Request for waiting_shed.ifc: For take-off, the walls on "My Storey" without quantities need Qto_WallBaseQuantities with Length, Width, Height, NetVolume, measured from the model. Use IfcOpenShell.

First a look at what the model holds.

```python
import ifcopenshell
import ifcopenshell.util.element
import ifcopenshell.util.unit

model = ifcopenshell.open("waiting_shed.ifc")
print(model.schema)
for unit_type in ("LENGTHUNIT", "AREAUNIT", "VOLUMEUNIT"):
    print(unit_type, ifcopenshell.util.unit.calculate_unit_scale(model, unit_type))
storey = next(s for s in model.by_type("IfcBuildingStorey") if s.Name == "My Storey")
walls = [e for e in ifcopenshell.util.element.get_decomposition(storey) if e.is_a("IfcWall")]
for e in sorted(walls, key=lambda e: e.id()):
    print(e.id(), e.is_a(), e.Name, list(ifcopenshell.util.element.get_psets(e, qtos_only=True)), sep=" | ")
```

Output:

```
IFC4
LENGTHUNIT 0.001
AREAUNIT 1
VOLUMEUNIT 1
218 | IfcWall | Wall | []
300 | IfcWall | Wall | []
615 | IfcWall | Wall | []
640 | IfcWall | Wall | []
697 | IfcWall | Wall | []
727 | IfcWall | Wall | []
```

```python
import ifcopenshell
import ifcopenshell.api.pset
import ifcopenshell.geom
import ifcopenshell.util.element
import ifcopenshell.util.shape
import ifcopenshell.util.unit

model = ifcopenshell.open("waiting_shed.ifc")
unit_scale = ifcopenshell.util.unit.calculate_unit_scale(model)
volume_scale = ifcopenshell.util.unit.calculate_unit_scale(model, "VOLUMEUNIT")
settings = ifcopenshell.geom.settings()

storey = next(s for s in model.by_type("IfcBuildingStorey") if s.Name == "My Storey")
walls = [e for e in ifcopenshell.util.element.get_decomposition(storey) if e.is_a("IfcWall")]

for e in sorted(walls, key=lambda e: e.id()):
    if ifcopenshell.util.element.get_psets(e, qtos_only=True, should_inherit=False):
        continue
    # Geometry comes back in metres, in the element's own axes.
    shape = ifcopenshell.geom.create_shape(settings, e)
    values = {
        "Length": ifcopenshell.util.shape.get_x(shape.geometry) / unit_scale,
        "Width": ifcopenshell.util.shape.get_y(shape.geometry) / unit_scale,
        "Height": ifcopenshell.util.shape.get_z(shape.geometry) / unit_scale,
        "NetVolume": ifcopenshell.util.shape.get_volume(shape.geometry) / volume_scale,
    }
    qto = ifcopenshell.api.pset.add_qto(model, product=e, name="Qto_WallBaseQuantities")
    ifcopenshell.api.pset.edit_qto(model, qto=qto, properties=values)
    print(e.id(), {k: round(v, 3) for k, v in values.items()})

model.write("waiting_shed_v2.ifc")
```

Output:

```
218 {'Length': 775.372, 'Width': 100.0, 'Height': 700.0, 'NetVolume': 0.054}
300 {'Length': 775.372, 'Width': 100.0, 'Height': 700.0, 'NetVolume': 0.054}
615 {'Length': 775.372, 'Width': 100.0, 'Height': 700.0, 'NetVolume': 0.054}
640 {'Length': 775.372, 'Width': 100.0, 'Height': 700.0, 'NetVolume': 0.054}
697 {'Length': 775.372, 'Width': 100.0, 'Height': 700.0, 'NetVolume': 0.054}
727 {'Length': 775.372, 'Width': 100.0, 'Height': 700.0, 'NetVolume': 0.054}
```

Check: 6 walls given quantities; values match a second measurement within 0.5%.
